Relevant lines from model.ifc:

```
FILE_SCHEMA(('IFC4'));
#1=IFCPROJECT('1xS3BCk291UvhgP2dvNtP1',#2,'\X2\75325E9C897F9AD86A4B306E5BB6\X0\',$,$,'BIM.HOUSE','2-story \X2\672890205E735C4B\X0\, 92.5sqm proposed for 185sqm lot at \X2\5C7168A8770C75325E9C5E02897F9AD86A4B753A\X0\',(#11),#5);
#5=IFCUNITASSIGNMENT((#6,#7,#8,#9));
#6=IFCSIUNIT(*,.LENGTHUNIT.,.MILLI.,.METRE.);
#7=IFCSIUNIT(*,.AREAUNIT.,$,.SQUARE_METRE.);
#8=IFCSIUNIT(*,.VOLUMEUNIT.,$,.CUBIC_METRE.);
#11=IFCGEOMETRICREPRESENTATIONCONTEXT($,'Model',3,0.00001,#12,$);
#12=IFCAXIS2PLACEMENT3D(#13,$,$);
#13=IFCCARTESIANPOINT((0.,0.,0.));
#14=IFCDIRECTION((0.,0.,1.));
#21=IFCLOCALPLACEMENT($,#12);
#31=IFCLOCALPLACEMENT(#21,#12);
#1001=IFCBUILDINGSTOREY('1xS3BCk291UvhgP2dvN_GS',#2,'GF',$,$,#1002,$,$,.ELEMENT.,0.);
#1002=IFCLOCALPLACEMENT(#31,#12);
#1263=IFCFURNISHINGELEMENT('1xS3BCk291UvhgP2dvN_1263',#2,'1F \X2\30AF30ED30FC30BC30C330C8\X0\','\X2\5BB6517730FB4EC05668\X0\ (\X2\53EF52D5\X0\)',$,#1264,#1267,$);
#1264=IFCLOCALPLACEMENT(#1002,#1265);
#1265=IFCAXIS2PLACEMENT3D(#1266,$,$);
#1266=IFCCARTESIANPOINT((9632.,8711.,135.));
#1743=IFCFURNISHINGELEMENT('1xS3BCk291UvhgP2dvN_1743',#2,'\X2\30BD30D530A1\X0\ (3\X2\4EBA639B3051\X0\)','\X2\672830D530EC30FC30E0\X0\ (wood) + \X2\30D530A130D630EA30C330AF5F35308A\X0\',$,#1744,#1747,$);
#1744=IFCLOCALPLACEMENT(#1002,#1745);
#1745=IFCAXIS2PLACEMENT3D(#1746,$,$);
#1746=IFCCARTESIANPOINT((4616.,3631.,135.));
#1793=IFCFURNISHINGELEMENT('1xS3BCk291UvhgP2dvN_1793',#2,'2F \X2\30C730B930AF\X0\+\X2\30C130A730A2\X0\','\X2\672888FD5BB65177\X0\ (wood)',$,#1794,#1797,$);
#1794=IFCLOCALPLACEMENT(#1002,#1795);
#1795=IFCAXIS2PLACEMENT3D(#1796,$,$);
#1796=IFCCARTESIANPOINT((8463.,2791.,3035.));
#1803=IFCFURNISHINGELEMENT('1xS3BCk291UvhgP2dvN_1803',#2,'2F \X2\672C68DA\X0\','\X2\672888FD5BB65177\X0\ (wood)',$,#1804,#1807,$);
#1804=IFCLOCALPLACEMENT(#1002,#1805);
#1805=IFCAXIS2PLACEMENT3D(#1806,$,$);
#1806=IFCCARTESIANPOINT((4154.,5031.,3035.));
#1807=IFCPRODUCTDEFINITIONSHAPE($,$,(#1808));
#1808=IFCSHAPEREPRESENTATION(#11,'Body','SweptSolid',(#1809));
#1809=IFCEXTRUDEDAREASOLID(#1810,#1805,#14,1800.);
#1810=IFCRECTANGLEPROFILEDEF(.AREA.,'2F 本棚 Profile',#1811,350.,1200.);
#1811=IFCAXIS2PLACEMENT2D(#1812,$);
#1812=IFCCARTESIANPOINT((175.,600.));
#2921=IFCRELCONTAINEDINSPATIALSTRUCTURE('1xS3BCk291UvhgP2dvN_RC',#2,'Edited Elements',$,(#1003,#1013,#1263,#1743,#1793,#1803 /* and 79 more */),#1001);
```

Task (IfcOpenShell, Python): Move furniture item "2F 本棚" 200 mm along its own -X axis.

```python
import ifcopenshell
import ifcopenshell.api.geometry
import ifcopenshell.util.placement

model = ifcopenshell.open("model.ifc")

item = model.by_guid("1xS3BCk291UvhgP2dvN_1803")
matrix = ifcopenshell.util.placement.get_local_placement(item.ObjectPlacement)
matrix[:3, 3] -= matrix[:3, 0] * 200.0
ifcopenshell.api.geometry.edit_object_placement(model, product=item, matrix=matrix, is_si=False)

print(ifcopenshell.util.placement.get_local_placement(item.ObjectPlacement).round(3) + 0.0)

model.write("model_rev.ifc")
```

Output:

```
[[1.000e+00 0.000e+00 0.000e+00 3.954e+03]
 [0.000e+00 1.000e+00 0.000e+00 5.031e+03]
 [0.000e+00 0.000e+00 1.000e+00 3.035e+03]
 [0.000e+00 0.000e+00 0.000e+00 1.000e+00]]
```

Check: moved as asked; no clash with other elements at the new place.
